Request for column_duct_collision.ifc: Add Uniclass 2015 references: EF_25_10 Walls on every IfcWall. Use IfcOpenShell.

First a look at what the model holds.

```python
import ifcopenshell

model = ifcopenshell.open("column_duct_collision.ifc")
print(model.schema)
print("classifications:", [c.Name for c in model.by_type("IfcClassification")])
for ifc_class in ("IfcDoor", "IfcRoof", "IfcStair", "IfcWall", "IfcWindow"):
    print(ifc_class, len(model.by_type(ifc_class)))
```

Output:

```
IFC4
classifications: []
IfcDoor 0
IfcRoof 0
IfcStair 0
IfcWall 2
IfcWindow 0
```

```python
import ifcopenshell
import ifcopenshell.api.classification

model = ifcopenshell.open("column_duct_collision.ifc")

system = ifcopenshell.api.classification.add_classification(model, classification="Uniclass 2015")

codes = {
    "IfcWall": ("EF_25_10", "Walls"),
}
for ifc_class, (code, name) in codes.items():
    products = model.by_type(ifc_class)
    ifcopenshell.api.classification.add_reference(
        model, products=products, classification=system, identification=code, name=name
    )
    print(code, len(products))

model.write("column_duct_collision_updated.ifc")
```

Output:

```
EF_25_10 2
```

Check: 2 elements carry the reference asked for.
